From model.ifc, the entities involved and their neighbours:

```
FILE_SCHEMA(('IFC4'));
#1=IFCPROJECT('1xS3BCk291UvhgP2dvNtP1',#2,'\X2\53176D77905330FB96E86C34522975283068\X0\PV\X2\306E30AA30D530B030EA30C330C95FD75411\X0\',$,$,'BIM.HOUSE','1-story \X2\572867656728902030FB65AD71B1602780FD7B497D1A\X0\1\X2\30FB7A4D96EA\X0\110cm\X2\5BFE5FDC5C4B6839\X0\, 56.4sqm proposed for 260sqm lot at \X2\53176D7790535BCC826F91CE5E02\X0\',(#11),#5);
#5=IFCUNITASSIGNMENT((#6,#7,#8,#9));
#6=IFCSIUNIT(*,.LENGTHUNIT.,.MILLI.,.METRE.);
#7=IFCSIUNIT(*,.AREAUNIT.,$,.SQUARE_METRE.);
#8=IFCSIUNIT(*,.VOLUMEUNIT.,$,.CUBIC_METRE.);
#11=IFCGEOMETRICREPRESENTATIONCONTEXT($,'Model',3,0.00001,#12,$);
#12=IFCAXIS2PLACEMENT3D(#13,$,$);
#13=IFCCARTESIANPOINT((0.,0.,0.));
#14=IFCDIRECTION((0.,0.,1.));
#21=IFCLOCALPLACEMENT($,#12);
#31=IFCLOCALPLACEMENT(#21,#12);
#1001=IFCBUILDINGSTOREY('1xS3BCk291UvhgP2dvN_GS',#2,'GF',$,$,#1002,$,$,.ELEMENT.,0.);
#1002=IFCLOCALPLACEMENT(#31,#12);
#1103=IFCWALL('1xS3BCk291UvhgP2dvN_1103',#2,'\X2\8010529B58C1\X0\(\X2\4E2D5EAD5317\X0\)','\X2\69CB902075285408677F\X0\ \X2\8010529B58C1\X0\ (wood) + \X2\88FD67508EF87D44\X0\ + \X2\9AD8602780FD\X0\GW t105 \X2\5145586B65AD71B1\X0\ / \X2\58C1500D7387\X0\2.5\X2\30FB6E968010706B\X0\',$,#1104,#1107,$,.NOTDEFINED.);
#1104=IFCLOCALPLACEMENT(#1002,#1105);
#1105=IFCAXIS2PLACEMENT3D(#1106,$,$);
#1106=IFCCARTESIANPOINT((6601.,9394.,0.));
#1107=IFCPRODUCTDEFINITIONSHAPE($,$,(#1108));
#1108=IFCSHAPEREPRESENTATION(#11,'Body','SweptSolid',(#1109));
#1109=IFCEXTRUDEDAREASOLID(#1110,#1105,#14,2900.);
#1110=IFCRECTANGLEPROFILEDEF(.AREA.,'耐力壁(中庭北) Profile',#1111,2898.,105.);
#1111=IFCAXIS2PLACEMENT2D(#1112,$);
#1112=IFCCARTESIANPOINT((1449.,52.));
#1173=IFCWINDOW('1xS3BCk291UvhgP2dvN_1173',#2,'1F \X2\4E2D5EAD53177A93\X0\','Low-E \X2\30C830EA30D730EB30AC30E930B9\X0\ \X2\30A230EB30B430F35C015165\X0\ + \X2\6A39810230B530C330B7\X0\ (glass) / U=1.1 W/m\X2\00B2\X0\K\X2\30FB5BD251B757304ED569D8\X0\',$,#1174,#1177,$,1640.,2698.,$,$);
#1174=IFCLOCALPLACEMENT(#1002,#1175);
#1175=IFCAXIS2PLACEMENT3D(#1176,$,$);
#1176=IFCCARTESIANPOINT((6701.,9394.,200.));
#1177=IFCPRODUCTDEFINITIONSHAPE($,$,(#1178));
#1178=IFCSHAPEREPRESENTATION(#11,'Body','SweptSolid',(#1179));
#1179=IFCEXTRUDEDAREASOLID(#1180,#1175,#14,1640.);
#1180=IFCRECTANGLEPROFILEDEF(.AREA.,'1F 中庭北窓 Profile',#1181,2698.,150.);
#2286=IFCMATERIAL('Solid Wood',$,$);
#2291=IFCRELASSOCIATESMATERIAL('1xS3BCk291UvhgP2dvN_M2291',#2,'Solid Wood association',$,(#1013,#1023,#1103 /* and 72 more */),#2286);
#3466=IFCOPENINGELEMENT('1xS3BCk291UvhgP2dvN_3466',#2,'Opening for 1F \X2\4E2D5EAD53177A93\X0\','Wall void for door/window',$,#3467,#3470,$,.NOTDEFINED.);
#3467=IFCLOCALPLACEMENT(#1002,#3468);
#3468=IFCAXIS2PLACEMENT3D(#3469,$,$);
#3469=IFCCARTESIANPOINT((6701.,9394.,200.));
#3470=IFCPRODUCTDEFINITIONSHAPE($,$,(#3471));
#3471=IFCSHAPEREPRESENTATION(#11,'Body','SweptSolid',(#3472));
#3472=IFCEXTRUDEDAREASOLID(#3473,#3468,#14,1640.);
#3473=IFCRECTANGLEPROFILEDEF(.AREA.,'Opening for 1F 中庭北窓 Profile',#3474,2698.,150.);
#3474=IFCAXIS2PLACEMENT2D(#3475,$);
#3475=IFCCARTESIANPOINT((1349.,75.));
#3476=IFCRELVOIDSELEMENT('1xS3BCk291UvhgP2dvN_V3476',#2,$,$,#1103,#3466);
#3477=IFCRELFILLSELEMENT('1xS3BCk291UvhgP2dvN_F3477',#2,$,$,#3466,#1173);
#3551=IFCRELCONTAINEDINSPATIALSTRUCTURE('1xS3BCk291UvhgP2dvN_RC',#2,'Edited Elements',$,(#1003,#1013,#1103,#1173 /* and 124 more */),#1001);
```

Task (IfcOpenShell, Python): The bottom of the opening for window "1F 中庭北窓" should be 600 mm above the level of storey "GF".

```python
import numpy as np
import ifcopenshell
import ifcopenshell.api.geometry
import ifcopenshell.geom
import ifcopenshell.util.element
import ifcopenshell.util.placement
import ifcopenshell.util.shape
import ifcopenshell.util.unit

model = ifcopenshell.open("model.ifc")
unit_scale = ifcopenshell.util.unit.calculate_unit_scale(model)

window = model.by_guid("1xS3BCk291UvhgP2dvN_1173")
opening = window.FillsVoids[0].RelatingOpeningElement
storey = ifcopenshell.util.element.get_container(window, ifc_class="IfcBuildingStorey")
level = ifcopenshell.util.placement.get_local_placement(storey.ObjectPlacement)[2, 3]

# The opening's origin need not be at the sill, so measure its lowest point.
shape = ifcopenshell.geom.create_shape(ifcopenshell.geom.settings(), opening)
bottom = ifcopenshell.util.shape.get_shape_bottom_elevation(shape, shape.geometry) / unit_scale
dz = level + 0.6 / unit_scale - bottom

shift = np.array([0.0, 0.0, dz])
# The window is not placed relative to its opening, so move both.
for product in (opening, window):
    matrix = ifcopenshell.util.placement.get_local_placement(product.ObjectPlacement)
    matrix[:3, 3] += shift
    ifcopenshell.api.geometry.edit_object_placement(model, product=product, matrix=matrix, is_si=False)

print(f"moved by {dz * unit_scale:+.3f} m")

model.write("model_edited.ifc")
```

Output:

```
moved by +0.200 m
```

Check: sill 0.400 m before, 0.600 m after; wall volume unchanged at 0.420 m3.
